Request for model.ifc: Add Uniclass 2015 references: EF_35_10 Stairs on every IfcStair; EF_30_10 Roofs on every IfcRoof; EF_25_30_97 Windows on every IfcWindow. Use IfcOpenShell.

First a look at what the model holds.

```python
import ifcopenshell

model = ifcopenshell.open("model.ifc")
print(model.schema)
print("classifications:", [c.Name for c in model.by_type("IfcClassification")])
for ifc_class in ("IfcDoor", "IfcRoof", "IfcStair", "IfcWall", "IfcWindow"):
    print(ifc_class, len(model.by_type(ifc_class)))
```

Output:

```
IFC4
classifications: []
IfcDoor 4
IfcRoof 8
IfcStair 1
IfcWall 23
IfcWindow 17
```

```python
import ifcopenshell
import ifcopenshell.api.classification

model = ifcopenshell.open("model.ifc")

system = ifcopenshell.api.classification.add_classification(model, classification="Uniclass 2015")

codes = {
    "IfcStair": ("EF_35_10", "Stairs"),
    "IfcRoof": ("EF_30_10", "Roofs"),
    "IfcWindow": ("EF_25_30_97", "Windows"),
}
for ifc_class, (code, name) in codes.items():
    products = model.by_type(ifc_class)
    ifcopenshell.api.classification.add_reference(
        model, products=products, classification=system, identification=code, name=name
    )
    print(code, len(products))

model.write("model_v2.ifc")
```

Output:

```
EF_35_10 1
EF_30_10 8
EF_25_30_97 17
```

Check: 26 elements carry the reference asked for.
